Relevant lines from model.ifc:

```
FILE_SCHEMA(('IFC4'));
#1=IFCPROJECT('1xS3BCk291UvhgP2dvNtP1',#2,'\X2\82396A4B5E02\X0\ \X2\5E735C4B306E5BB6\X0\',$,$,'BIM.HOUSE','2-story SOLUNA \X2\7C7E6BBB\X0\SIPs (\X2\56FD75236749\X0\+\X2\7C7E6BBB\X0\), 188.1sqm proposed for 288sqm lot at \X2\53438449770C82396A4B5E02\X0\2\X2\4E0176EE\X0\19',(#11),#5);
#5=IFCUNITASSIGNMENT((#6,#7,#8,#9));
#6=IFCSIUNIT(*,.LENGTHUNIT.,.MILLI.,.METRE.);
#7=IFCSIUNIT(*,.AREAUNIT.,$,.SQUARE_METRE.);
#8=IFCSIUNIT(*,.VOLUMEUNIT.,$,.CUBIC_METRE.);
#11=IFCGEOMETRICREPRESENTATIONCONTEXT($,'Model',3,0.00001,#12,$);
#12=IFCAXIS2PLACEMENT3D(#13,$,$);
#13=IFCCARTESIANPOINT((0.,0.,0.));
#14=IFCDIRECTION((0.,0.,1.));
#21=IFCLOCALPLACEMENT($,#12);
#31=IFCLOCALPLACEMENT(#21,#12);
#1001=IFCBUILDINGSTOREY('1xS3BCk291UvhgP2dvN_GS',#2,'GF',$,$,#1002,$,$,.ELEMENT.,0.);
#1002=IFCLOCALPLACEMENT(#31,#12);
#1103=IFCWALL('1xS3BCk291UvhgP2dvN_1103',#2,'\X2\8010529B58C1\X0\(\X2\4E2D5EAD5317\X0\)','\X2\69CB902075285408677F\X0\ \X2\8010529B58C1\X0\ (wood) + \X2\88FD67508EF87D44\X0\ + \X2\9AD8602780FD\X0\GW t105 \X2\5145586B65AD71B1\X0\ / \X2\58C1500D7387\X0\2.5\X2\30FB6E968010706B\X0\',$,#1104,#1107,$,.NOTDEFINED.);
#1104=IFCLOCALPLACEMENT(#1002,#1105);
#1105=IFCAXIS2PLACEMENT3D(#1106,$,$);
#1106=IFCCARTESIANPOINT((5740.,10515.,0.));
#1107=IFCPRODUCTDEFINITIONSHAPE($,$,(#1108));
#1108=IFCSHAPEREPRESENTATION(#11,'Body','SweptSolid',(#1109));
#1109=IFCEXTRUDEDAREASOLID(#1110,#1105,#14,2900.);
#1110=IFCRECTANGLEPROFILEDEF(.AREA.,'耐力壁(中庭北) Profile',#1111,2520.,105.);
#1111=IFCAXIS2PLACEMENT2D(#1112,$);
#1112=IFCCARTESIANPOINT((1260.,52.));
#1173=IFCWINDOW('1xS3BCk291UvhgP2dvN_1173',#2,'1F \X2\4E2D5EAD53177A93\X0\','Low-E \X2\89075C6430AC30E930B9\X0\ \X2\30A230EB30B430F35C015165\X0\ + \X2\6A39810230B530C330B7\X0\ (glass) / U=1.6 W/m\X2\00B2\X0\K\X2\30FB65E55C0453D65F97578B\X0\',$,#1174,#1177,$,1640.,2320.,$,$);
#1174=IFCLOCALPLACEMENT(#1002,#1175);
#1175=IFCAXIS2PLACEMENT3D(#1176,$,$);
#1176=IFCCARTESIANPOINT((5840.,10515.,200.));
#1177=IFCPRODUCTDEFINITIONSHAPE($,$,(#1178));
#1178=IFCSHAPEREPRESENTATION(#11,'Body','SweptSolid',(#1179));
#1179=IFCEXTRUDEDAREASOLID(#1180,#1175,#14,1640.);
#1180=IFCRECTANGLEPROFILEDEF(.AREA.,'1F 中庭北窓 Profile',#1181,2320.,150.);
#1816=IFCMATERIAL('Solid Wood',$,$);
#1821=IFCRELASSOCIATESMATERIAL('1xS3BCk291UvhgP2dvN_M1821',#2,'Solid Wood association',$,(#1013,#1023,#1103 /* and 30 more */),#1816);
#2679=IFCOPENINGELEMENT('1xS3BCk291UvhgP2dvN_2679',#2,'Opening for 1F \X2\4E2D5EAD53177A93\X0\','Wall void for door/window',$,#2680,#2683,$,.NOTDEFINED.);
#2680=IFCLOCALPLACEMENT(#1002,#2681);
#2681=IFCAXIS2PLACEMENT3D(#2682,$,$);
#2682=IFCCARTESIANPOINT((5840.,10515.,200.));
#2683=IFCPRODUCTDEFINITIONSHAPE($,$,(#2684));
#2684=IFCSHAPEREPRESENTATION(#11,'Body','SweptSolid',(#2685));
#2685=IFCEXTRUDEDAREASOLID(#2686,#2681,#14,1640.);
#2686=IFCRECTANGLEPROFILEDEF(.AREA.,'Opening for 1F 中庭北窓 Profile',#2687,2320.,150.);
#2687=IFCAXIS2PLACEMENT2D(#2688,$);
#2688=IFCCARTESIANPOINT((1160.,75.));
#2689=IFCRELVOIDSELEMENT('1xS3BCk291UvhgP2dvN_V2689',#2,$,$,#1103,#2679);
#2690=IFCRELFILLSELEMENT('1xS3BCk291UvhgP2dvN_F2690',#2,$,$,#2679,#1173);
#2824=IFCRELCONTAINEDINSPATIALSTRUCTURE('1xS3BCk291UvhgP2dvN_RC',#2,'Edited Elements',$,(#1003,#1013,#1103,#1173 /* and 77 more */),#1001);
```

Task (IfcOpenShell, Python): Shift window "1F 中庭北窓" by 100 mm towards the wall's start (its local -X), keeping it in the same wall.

```python
import ifcopenshell
import ifcopenshell.api.geometry
import ifcopenshell.util.placement
import ifcopenshell.util.unit

model = ifcopenshell.open("model.ifc")
unit_scale = ifcopenshell.util.unit.calculate_unit_scale(model)

window = model.by_id(1173)
opening = window.FillsVoids[0].RelatingOpeningElement
wall = opening.VoidsElements[0].RelatingBuildingElement

wall_matrix = ifcopenshell.util.placement.get_local_placement(wall.ObjectPlacement)
shift = wall_matrix[:3, 0] * -0.1 / unit_scale
before = ifcopenshell.util.placement.get_local_placement(window.ObjectPlacement)[:3, 3].copy()

# The window is not placed relative to its opening, so move both.
for product in (opening, window):
    matrix = ifcopenshell.util.placement.get_local_placement(product.ObjectPlacement)
    matrix[:3, 3] += shift
    ifcopenshell.api.geometry.edit_object_placement(model, product=product, matrix=matrix, is_si=False)

after = ifcopenshell.util.placement.get_local_placement(window.ObjectPlacement)[:3, 3]
print("window moved by", (after - before).round(3) + 0.0)

model.write("model-out.ifc")
```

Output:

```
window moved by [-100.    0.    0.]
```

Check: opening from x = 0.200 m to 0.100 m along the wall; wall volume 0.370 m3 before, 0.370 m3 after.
